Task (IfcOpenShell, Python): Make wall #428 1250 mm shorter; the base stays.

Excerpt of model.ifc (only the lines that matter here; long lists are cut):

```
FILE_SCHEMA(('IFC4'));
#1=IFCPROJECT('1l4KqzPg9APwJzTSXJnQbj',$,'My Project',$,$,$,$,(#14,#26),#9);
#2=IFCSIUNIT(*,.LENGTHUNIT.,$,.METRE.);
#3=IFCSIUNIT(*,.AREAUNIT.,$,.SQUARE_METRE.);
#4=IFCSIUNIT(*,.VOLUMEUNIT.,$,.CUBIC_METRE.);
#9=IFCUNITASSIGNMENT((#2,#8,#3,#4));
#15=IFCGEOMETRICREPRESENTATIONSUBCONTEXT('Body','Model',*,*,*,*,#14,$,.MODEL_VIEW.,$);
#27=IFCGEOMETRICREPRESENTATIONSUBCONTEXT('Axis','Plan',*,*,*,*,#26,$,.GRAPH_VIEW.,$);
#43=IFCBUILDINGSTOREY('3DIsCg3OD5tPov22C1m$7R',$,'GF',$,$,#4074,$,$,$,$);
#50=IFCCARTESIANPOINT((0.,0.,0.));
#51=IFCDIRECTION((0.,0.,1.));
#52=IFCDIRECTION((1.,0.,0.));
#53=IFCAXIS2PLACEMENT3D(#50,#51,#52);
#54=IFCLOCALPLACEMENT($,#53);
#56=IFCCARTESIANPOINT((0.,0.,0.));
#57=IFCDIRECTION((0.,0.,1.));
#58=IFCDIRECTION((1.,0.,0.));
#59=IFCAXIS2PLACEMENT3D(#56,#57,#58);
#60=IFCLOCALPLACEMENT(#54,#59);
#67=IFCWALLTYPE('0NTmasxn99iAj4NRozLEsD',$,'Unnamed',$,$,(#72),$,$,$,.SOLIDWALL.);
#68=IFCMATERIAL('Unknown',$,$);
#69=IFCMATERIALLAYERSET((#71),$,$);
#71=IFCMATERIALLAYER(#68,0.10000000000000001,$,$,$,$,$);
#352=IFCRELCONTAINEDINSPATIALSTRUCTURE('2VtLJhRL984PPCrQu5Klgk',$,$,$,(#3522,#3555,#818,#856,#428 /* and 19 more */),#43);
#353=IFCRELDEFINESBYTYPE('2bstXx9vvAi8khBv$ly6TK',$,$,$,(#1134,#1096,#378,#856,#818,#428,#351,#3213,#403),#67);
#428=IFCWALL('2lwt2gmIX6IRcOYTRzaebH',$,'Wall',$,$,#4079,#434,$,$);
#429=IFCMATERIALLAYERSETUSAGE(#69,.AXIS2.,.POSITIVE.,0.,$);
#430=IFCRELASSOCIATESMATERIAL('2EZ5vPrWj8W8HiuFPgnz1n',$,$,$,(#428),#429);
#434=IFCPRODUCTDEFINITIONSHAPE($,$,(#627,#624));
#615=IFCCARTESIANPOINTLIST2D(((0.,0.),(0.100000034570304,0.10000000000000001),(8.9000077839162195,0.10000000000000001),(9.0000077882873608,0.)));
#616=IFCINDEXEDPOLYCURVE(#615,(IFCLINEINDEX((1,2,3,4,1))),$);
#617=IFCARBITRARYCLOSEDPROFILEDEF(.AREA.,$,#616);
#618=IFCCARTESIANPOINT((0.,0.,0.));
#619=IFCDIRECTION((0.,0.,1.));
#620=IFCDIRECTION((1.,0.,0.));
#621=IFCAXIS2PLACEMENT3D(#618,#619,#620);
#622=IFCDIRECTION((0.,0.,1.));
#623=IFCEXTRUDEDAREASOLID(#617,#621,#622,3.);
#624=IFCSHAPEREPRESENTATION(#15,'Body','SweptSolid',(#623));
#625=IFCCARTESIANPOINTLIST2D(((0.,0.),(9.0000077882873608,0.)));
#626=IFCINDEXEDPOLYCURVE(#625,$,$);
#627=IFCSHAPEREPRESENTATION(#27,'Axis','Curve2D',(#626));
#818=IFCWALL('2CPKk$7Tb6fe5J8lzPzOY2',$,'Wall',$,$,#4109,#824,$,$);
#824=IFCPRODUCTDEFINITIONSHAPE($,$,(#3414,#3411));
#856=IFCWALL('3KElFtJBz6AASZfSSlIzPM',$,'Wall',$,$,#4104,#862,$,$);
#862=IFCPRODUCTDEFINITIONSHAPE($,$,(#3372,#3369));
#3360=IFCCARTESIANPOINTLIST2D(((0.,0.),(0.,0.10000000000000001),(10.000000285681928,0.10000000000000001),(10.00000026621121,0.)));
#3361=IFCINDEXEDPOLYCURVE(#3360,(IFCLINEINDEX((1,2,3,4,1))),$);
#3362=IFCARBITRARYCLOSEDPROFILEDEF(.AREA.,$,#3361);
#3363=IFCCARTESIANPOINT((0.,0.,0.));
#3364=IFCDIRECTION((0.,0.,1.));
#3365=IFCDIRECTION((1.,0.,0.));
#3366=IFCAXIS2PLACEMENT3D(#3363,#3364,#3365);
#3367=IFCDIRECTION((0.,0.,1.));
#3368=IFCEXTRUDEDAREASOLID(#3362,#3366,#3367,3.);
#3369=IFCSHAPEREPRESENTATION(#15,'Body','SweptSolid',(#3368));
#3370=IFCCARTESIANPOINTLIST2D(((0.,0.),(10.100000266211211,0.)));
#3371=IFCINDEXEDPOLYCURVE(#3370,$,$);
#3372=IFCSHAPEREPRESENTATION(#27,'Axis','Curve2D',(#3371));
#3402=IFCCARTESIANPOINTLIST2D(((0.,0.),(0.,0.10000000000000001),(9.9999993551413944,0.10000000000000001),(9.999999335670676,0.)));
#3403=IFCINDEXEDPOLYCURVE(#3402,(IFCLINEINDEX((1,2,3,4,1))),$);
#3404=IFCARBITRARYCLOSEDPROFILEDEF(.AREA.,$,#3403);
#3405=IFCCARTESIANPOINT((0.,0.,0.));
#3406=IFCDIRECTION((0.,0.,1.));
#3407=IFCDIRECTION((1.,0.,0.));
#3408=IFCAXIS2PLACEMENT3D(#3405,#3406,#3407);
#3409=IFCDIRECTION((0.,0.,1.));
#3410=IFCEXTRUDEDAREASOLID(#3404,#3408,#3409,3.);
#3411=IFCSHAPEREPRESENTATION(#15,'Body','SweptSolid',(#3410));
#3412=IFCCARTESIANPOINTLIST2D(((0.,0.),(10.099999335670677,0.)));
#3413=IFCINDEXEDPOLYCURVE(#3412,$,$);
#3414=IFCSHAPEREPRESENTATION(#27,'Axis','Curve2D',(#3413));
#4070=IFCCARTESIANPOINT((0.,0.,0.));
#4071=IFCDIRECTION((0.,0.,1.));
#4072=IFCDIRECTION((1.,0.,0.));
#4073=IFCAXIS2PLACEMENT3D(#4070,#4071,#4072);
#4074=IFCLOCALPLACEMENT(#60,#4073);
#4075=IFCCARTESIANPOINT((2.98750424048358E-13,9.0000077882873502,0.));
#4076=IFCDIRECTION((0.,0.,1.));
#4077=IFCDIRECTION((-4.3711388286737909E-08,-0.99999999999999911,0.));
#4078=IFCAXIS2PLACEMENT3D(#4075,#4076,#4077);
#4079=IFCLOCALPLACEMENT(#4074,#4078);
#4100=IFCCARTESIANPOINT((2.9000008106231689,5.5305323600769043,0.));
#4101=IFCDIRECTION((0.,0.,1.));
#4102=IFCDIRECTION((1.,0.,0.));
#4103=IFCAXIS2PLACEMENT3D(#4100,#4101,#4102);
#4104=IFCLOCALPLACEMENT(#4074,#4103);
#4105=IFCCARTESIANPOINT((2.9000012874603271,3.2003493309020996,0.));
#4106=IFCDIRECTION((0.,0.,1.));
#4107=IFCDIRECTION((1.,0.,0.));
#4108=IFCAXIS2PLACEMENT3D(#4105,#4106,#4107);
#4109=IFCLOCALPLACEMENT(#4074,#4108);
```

```python
import ifcopenshell
import ifcopenshell.geom
import ifcopenshell.util.representation
import ifcopenshell.util.shape
import ifcopenshell.util.unit

model = ifcopenshell.open("model.ifc")
unit_scale = ifcopenshell.util.unit.calculate_unit_scale(model)
settings = ifcopenshell.geom.settings()


def volume(element):
    """Net volume in cubic metres, openings subtracted."""
    shape = ifcopenshell.geom.create_shape(settings, element)
    return ifcopenshell.util.shape.get_volume(shape.geometry)


wall = model.by_guid("2lwt2gmIX6IRcOYTRzaebH")
before = volume(wall)

body = ifcopenshell.util.representation.get_representation(wall, "Model", "Body")
solid = body.Items[0]
old_height = solid.Depth
solid.Depth -= 1.25 / unit_scale
after = volume(wall)

print(f"height {old_height:g} -> {solid.Depth:g}, volume {before:.3f} -> {after:.3f} m3")

model.write("model-out.ifc")
```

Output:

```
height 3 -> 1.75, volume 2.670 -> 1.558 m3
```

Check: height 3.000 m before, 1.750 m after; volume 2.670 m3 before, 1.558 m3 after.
